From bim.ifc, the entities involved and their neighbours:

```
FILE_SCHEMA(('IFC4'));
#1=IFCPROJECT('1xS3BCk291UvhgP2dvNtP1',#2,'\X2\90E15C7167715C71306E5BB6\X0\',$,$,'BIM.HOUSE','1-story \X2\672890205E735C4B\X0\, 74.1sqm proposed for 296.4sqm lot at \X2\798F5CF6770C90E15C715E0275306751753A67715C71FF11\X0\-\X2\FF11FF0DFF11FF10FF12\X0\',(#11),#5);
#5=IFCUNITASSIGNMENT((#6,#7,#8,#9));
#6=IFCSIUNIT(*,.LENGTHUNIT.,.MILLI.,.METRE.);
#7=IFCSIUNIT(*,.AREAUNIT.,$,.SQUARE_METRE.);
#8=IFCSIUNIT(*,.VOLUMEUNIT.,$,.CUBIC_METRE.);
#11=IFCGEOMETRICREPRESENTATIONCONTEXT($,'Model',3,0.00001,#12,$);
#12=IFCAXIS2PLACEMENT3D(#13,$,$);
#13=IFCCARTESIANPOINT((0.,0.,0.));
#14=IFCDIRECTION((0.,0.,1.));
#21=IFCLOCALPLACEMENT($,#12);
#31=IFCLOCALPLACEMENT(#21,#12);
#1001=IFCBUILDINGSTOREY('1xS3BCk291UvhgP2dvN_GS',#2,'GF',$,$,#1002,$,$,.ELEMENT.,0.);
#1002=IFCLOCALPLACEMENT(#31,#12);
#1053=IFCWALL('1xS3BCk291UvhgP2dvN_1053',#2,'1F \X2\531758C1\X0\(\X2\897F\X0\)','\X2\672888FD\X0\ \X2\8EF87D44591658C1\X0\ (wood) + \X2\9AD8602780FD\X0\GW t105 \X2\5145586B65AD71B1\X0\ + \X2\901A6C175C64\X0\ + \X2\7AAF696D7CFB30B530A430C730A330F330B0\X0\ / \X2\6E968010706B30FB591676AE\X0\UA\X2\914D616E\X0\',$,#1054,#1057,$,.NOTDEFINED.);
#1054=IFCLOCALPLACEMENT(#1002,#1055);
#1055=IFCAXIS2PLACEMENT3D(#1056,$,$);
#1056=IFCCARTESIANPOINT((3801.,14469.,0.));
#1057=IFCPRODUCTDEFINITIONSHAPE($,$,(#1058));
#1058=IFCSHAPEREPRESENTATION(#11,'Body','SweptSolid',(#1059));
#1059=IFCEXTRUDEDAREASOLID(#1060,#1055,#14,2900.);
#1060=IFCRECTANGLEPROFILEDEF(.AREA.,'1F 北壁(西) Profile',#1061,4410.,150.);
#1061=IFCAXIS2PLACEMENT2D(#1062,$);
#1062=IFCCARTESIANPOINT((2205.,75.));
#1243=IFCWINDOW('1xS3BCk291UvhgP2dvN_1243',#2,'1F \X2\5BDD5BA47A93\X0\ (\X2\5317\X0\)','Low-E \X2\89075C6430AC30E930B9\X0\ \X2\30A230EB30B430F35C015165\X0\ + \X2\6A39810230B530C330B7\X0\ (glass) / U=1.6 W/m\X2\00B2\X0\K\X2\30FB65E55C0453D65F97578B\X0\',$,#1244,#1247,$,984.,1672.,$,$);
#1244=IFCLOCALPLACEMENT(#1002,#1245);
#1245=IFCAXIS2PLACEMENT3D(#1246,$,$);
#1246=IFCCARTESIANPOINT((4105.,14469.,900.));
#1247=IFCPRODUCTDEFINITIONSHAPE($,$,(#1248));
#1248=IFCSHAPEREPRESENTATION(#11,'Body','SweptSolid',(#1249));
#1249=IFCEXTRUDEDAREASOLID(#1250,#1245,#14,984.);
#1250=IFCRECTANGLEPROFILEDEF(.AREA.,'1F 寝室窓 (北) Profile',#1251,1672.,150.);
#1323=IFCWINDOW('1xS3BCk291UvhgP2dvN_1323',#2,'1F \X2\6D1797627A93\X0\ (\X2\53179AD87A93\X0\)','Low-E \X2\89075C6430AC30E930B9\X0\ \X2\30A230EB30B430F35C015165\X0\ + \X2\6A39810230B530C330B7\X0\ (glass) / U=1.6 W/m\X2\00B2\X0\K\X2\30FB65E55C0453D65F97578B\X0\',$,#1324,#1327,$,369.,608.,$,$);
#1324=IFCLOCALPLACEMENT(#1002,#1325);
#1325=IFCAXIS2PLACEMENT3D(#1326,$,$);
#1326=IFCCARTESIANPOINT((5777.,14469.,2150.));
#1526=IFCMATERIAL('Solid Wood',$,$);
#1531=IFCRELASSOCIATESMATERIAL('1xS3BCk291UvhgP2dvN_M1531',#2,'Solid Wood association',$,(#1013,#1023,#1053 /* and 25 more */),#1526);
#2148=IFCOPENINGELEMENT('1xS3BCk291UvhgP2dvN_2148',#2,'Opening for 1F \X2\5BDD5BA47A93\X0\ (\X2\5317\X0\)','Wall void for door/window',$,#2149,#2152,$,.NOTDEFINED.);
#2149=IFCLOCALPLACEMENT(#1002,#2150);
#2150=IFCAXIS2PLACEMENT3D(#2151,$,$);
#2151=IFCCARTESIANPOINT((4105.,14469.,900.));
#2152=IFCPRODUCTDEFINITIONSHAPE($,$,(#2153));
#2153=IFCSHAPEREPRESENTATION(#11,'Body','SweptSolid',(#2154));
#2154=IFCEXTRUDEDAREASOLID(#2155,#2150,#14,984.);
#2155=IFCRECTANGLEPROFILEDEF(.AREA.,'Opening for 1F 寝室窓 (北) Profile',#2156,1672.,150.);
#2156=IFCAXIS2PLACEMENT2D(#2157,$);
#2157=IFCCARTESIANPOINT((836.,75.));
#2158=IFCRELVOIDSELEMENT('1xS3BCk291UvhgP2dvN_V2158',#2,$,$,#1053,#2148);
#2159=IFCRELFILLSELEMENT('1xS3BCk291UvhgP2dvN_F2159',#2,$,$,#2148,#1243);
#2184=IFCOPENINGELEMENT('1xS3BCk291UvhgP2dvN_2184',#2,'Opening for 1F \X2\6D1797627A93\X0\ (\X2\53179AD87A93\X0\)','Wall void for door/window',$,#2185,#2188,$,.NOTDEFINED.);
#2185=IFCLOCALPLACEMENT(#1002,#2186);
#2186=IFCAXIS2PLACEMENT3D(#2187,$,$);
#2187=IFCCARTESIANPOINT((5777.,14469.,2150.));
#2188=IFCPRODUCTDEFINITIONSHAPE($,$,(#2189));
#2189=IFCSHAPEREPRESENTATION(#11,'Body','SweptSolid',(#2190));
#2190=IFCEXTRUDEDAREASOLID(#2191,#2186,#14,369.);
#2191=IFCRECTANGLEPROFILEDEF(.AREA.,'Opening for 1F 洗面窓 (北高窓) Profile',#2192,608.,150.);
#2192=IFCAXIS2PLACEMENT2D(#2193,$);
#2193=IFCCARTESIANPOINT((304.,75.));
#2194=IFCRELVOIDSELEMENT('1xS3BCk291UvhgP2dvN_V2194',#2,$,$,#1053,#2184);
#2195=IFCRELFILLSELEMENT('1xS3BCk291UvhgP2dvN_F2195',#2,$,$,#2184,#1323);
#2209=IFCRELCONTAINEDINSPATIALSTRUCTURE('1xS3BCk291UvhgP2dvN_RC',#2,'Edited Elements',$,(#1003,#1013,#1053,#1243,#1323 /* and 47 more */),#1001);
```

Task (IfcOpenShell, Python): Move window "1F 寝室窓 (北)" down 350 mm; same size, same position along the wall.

```python
import numpy as np
import ifcopenshell
import ifcopenshell.api.geometry
import ifcopenshell.util.placement
import ifcopenshell.util.unit

model = ifcopenshell.open("bim.ifc")
unit_scale = ifcopenshell.util.unit.calculate_unit_scale(model)

window = model.by_guid("1xS3BCk291UvhgP2dvN_1243")
opening = window.FillsVoids[0].RelatingOpeningElement
dz = -350.0

shift = np.array([0.0, 0.0, dz])
# The window is not placed relative to its opening, so move both.
for product in (opening, window):
    matrix = ifcopenshell.util.placement.get_local_placement(product.ObjectPlacement)
    matrix[:3, 3] += shift
    ifcopenshell.api.geometry.edit_object_placement(model, product=product, matrix=matrix, is_si=False)

print(f"moved by {dz * unit_scale:+.3f} m")

model.write("bim_v2.ifc")
```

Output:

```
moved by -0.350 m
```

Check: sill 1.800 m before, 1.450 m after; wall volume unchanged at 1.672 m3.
